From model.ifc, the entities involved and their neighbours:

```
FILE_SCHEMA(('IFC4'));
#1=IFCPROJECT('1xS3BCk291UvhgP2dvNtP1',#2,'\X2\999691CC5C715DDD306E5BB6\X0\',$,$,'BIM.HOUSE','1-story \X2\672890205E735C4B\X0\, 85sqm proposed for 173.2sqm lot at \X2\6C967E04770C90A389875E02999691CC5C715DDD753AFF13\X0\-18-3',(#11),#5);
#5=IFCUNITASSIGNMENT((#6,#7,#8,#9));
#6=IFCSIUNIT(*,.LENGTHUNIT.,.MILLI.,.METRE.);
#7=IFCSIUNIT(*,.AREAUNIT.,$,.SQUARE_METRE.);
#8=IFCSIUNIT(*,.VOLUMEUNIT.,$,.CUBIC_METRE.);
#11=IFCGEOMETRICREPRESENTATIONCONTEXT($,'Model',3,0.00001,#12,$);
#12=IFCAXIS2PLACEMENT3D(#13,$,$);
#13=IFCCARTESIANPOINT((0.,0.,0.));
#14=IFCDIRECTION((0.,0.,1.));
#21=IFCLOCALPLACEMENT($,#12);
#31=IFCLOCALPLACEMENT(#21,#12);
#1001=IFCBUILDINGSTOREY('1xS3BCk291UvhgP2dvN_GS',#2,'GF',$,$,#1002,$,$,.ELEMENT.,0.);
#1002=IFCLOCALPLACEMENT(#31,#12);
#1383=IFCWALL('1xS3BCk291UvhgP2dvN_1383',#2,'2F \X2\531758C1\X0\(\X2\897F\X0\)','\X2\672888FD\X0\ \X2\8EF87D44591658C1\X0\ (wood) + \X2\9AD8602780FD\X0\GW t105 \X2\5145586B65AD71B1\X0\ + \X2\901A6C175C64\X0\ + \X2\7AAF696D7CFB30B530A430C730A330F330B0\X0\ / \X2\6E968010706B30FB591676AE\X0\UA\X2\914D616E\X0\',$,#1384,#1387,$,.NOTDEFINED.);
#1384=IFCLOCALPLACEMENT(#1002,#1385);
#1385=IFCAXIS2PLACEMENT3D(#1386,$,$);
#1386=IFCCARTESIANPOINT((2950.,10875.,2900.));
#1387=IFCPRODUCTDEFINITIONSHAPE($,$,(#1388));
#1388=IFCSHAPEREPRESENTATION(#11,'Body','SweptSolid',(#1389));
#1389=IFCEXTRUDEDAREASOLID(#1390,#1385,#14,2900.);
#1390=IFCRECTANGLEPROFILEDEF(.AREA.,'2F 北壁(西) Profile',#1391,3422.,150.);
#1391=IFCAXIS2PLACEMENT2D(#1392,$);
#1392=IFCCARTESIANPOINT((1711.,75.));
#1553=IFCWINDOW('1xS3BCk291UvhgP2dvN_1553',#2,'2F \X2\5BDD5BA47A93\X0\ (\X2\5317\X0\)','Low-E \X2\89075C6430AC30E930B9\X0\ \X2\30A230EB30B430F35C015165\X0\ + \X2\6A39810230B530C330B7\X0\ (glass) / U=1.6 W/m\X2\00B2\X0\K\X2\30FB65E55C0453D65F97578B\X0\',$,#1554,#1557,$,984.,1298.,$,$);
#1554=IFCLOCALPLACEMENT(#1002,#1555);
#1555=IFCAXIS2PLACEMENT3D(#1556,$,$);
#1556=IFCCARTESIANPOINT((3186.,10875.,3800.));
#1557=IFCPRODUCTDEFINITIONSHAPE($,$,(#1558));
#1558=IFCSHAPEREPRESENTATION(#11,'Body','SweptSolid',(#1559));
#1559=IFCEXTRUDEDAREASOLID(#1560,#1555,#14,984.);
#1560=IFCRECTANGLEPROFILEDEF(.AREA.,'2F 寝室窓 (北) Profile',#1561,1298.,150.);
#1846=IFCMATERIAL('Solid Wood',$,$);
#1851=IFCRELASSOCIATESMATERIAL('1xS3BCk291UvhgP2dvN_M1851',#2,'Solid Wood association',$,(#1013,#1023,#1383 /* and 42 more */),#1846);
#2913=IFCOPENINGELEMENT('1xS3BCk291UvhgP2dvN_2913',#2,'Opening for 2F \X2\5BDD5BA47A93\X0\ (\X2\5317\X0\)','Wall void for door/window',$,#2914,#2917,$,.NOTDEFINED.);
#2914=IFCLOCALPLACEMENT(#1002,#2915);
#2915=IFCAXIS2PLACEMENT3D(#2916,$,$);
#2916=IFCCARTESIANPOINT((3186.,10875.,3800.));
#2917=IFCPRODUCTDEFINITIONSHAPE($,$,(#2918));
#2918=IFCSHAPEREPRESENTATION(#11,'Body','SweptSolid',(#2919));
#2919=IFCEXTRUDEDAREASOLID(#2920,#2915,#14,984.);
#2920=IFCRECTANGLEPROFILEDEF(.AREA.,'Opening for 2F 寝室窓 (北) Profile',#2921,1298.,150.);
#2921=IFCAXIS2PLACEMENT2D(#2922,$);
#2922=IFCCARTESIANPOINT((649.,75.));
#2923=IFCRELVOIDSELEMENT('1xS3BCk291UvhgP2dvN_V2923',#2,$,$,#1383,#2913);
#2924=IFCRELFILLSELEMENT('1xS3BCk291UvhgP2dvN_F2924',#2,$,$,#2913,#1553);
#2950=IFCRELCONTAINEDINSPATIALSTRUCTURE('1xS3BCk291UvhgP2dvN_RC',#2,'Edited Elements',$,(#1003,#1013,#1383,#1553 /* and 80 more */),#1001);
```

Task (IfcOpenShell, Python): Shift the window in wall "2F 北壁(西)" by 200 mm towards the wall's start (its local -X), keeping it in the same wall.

```python
import ifcopenshell
import ifcopenshell.api.geometry
import ifcopenshell.util.placement
import ifcopenshell.util.unit

model = ifcopenshell.open("model.ifc")
unit_scale = ifcopenshell.util.unit.calculate_unit_scale(model)

window = model.by_guid("1xS3BCk291UvhgP2dvN_1553")
opening = window.FillsVoids[0].RelatingOpeningElement
wall = opening.VoidsElements[0].RelatingBuildingElement

wall_matrix = ifcopenshell.util.placement.get_local_placement(wall.ObjectPlacement)
shift = wall_matrix[:3, 0] * -0.2 / unit_scale
before = ifcopenshell.util.placement.get_local_placement(window.ObjectPlacement)[:3, 3].copy()

# The window is not placed relative to its opening, so move both.
for product in (opening, window):
    matrix = ifcopenshell.util.placement.get_local_placement(product.ObjectPlacement)
    matrix[:3, 3] += shift
    ifcopenshell.api.geometry.edit_object_placement(model, product=product, matrix=matrix, is_si=False)

after = ifcopenshell.util.placement.get_local_placement(window.ObjectPlacement)[:3, 3]
print("window moved by", (after - before).round(3) + 0.0)

model.write("model_v2.ifc")
```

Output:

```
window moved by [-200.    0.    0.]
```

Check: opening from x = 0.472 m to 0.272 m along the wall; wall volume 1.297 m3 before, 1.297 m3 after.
